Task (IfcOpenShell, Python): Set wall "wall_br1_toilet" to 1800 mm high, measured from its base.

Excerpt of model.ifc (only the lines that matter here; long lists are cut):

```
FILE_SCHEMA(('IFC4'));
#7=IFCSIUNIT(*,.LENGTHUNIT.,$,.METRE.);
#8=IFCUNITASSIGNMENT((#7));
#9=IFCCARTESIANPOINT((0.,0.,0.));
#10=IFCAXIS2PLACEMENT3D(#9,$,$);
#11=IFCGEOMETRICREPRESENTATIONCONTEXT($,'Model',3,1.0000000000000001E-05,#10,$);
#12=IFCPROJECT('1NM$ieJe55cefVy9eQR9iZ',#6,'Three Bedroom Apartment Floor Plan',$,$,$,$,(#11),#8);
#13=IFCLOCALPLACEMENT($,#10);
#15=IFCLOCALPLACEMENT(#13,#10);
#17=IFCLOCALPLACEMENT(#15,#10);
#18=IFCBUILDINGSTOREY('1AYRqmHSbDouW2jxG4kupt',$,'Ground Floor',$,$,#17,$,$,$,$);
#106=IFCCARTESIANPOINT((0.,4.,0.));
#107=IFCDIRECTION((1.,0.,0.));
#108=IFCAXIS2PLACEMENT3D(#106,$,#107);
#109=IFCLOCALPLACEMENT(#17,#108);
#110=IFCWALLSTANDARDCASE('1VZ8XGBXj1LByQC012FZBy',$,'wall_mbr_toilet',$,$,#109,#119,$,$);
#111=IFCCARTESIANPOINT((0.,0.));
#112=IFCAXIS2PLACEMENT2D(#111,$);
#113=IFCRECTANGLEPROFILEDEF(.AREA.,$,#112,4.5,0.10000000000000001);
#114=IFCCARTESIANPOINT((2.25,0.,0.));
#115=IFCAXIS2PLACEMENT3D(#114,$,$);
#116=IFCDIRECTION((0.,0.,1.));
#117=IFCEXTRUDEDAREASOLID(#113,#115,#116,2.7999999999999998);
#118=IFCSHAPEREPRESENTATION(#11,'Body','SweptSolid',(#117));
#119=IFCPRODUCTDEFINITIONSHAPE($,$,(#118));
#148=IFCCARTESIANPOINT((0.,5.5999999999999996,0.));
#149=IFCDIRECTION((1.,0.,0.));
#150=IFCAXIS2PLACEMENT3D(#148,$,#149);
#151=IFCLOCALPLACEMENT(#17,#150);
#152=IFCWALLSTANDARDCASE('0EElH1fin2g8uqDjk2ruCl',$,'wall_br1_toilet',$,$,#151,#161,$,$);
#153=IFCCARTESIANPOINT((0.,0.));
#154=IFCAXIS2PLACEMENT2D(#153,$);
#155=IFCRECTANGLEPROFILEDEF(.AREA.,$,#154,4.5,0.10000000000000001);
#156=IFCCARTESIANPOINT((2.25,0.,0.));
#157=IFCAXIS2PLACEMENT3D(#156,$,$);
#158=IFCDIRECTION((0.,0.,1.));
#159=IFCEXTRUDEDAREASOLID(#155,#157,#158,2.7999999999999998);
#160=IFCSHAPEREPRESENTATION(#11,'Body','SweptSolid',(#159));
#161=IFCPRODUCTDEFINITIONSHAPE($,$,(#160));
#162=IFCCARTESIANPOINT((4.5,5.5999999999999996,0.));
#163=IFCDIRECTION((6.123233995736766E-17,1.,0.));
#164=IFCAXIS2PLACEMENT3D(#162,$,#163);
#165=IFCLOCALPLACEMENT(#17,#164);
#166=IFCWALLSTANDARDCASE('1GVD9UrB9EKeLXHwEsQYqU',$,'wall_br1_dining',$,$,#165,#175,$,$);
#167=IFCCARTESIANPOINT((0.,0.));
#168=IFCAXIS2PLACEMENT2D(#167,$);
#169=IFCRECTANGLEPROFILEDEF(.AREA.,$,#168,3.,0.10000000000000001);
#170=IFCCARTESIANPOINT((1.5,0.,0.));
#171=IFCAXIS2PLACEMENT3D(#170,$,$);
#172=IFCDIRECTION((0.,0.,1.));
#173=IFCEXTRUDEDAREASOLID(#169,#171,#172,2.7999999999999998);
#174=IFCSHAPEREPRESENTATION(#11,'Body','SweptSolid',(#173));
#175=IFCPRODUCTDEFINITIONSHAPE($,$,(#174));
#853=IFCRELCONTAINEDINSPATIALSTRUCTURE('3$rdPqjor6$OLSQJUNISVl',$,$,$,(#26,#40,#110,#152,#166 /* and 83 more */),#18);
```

```python
import ifcopenshell
import ifcopenshell.geom
import ifcopenshell.util.shape
import ifcopenshell.util.unit

model = ifcopenshell.open("model.ifc")
unit_scale = ifcopenshell.util.unit.calculate_unit_scale(model)
settings = ifcopenshell.geom.settings()


def volume(element):
    """Net volume in cubic metres, openings subtracted."""
    shape = ifcopenshell.geom.create_shape(settings, element)
    return ifcopenshell.util.shape.get_volume(shape.geometry)


wall = model.by_id(152)
before = volume(wall)

body = next(r for r in wall.Representation.Representations if r.RepresentationIdentifier == "Body")
solid = body.Items[0]
old_height = solid.Depth
solid.Depth = 1.8 / unit_scale
after = volume(wall)

print(f"height {old_height:g} -> {solid.Depth:g}, volume {before:.3f} -> {after:.3f} m3")

model.write("model_v2.ifc")
```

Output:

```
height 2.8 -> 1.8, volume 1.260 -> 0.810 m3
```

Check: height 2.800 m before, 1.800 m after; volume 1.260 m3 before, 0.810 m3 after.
